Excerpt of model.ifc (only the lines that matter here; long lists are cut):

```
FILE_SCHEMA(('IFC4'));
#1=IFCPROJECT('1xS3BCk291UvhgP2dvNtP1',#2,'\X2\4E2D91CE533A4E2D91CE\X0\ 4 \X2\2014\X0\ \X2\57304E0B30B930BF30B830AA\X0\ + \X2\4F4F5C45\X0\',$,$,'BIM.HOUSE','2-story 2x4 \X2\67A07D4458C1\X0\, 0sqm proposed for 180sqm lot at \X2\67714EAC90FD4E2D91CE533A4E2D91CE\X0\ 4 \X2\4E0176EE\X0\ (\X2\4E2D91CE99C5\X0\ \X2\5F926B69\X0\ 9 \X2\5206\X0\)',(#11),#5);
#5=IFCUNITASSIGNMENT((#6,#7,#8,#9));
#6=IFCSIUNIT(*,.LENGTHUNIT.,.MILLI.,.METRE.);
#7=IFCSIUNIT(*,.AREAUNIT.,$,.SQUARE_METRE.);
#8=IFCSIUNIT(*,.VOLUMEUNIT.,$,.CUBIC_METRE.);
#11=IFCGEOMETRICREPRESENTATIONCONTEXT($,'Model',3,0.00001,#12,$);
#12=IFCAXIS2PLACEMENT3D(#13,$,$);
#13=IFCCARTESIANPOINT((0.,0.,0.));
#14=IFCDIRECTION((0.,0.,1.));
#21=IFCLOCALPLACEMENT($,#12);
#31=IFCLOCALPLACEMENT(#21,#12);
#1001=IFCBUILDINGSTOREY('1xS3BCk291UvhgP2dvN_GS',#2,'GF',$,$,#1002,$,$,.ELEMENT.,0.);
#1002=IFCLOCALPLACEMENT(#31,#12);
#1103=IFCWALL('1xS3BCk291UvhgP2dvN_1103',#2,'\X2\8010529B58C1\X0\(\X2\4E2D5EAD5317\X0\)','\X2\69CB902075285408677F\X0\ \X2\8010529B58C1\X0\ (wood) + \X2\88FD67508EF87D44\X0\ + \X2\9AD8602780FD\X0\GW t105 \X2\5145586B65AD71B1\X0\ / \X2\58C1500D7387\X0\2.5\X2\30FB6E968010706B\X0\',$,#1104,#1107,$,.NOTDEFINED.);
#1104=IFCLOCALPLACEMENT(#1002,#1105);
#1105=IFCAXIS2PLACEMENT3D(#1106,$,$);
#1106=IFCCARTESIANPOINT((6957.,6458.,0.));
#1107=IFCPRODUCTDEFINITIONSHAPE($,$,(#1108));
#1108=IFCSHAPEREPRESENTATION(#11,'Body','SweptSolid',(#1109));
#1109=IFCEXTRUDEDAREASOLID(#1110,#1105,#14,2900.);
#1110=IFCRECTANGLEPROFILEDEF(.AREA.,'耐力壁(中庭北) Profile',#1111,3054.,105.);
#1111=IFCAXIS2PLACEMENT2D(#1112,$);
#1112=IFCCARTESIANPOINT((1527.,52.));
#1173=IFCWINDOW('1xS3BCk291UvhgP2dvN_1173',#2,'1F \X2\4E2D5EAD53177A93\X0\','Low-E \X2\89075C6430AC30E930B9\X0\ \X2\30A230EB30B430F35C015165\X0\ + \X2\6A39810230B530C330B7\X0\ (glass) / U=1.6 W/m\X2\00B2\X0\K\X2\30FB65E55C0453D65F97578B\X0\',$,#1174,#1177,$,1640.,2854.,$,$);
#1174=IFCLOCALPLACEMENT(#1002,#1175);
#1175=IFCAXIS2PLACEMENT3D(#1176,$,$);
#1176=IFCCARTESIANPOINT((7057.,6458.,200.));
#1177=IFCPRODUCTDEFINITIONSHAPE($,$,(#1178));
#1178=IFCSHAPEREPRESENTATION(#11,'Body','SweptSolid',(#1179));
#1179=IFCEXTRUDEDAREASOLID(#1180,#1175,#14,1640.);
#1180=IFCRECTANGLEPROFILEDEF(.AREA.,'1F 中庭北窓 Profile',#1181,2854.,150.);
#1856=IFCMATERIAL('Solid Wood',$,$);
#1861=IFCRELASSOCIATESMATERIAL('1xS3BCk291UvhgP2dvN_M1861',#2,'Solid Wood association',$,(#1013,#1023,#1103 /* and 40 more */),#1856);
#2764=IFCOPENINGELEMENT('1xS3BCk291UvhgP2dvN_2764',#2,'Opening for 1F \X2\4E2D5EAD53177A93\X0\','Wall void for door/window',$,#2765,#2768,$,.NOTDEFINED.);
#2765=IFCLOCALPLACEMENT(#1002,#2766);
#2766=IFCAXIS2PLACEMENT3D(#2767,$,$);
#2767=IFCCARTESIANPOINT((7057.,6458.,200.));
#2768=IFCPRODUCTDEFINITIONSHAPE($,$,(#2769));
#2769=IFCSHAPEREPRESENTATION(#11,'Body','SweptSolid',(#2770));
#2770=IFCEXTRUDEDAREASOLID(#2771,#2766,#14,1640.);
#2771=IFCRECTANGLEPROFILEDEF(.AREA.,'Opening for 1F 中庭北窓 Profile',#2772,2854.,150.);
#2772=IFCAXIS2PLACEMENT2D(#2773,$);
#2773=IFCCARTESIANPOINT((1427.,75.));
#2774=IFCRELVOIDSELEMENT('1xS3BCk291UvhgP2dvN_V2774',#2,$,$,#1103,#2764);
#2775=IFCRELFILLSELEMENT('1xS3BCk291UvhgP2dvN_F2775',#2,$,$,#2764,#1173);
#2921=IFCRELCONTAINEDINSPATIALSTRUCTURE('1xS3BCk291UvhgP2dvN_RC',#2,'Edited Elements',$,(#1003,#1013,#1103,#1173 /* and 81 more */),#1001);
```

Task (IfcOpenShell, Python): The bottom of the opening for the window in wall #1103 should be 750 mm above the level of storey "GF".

```python
import numpy as np
import ifcopenshell
import ifcopenshell.api.geometry
import ifcopenshell.geom
import ifcopenshell.util.element
import ifcopenshell.util.placement
import ifcopenshell.util.shape
import ifcopenshell.util.unit

model = ifcopenshell.open("model.ifc")
unit_scale = ifcopenshell.util.unit.calculate_unit_scale(model)

window = model.by_guid("1xS3BCk291UvhgP2dvN_1173")
opening = window.FillsVoids[0].RelatingOpeningElement
storey = ifcopenshell.util.element.get_container(window, ifc_class="IfcBuildingStorey")
level = ifcopenshell.util.placement.get_local_placement(storey.ObjectPlacement)[2, 3]

# The opening's origin need not be at the sill, so measure its lowest point.
shape = ifcopenshell.geom.create_shape(ifcopenshell.geom.settings(), opening)
bottom = ifcopenshell.util.shape.get_shape_bottom_elevation(shape, shape.geometry) / unit_scale
dz = level + 750.0 - bottom

shift = np.array([0.0, 0.0, dz])
# The window is not placed relative to its opening, so move both.
for product in (opening, window):
    matrix = ifcopenshell.util.placement.get_local_placement(product.ObjectPlacement)
    matrix[:3, 3] += shift
    ifcopenshell.api.geometry.edit_object_placement(model, product=product, matrix=matrix, is_si=False)

print(f"moved by {dz * unit_scale:+.3f} m")

model.write("model_v2.ifc")
```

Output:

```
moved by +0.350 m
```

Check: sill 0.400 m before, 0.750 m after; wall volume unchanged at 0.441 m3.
